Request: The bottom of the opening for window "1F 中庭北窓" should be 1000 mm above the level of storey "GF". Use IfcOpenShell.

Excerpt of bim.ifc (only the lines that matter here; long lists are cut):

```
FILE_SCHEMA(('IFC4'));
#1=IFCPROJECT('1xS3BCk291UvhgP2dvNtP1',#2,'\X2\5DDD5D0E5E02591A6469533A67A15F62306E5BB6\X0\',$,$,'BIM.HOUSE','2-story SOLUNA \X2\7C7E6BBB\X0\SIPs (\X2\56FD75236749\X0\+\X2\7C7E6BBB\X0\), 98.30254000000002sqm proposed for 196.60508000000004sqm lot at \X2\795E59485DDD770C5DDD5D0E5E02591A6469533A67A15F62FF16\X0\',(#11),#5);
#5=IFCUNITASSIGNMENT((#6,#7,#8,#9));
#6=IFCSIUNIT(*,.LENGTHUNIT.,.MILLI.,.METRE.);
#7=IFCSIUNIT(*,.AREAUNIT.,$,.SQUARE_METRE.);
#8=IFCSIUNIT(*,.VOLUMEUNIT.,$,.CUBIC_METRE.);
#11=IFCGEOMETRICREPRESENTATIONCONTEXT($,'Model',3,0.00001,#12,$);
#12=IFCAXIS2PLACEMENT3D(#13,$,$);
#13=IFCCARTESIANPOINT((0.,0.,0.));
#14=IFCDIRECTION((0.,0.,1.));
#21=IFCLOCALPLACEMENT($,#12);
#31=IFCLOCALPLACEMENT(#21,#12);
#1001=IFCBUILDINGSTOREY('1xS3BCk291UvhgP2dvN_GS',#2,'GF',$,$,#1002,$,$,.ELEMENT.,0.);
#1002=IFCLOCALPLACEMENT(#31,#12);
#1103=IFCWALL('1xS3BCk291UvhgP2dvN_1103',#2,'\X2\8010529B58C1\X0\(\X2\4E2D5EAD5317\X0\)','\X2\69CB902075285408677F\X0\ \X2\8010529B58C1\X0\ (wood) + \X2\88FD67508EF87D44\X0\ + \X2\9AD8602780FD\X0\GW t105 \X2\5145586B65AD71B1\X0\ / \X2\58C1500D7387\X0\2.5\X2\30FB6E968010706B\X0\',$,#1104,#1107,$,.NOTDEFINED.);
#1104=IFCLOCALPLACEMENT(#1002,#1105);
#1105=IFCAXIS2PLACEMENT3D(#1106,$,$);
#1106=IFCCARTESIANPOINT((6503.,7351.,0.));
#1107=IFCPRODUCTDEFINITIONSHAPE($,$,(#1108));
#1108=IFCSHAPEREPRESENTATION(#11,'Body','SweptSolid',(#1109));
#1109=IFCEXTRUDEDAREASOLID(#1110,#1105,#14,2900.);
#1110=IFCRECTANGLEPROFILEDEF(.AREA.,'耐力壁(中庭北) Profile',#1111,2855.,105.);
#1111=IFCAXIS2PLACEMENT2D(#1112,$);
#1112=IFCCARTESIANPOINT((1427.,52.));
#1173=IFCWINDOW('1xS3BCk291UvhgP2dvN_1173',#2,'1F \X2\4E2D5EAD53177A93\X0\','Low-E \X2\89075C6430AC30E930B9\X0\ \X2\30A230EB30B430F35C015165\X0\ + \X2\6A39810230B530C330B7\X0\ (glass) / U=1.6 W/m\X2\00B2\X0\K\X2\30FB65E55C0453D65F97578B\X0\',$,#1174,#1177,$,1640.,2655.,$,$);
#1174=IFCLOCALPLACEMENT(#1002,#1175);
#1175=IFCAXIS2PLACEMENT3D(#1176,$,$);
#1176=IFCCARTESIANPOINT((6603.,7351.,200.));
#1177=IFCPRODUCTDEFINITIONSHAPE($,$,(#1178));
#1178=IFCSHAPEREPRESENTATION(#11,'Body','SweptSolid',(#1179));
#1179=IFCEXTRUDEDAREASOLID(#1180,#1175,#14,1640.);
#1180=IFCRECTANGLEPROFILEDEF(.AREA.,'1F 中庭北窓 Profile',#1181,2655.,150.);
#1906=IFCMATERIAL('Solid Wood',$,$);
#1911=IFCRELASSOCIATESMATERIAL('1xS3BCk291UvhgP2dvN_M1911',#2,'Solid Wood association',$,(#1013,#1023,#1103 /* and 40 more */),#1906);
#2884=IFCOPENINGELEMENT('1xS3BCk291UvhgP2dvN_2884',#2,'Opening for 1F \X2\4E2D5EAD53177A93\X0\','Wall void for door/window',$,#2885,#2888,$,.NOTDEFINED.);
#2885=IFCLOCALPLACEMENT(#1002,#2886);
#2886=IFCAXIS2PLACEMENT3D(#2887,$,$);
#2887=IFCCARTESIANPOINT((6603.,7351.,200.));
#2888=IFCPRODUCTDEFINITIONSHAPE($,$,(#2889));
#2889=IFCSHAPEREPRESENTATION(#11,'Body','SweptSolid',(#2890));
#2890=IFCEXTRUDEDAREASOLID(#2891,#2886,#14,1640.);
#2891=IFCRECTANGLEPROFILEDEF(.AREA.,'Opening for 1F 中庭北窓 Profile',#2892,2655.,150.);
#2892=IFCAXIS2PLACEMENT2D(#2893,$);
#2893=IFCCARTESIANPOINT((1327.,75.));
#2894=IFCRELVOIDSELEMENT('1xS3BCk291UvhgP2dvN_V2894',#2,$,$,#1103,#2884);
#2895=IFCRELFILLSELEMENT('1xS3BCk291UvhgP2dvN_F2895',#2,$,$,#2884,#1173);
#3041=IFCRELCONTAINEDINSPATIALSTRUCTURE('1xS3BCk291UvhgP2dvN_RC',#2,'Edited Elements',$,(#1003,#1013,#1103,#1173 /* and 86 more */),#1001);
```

```python
import numpy as np
import ifcopenshell
import ifcopenshell.api.geometry
import ifcopenshell.geom
import ifcopenshell.util.element
import ifcopenshell.util.placement
import ifcopenshell.util.shape
import ifcopenshell.util.unit

model = ifcopenshell.open("bim.ifc")
unit_scale = ifcopenshell.util.unit.calculate_unit_scale(model)

window = model.by_guid("1xS3BCk291UvhgP2dvN_1173")
opening = window.FillsVoids[0].RelatingOpeningElement
storey = ifcopenshell.util.element.get_container(window, ifc_class="IfcBuildingStorey")
level = ifcopenshell.util.placement.get_local_placement(storey.ObjectPlacement)[2, 3]

# The opening's origin need not be at the sill, so measure its lowest point.
shape = ifcopenshell.geom.create_shape(ifcopenshell.geom.settings(), opening)
bottom = ifcopenshell.util.shape.get_shape_bottom_elevation(shape, shape.geometry) / unit_scale
dz = level + 1 / unit_scale - bottom

shift = np.array([0.0, 0.0, dz])
# The window is not placed relative to its opening, so move both.
for product in (opening, window):
    matrix = ifcopenshell.util.placement.get_local_placement(product.ObjectPlacement)
    matrix[:3, 3] += shift
    ifcopenshell.api.geometry.edit_object_placement(model, product=product, matrix=matrix, is_si=False)

print(f"moved by {dz * unit_scale:+.3f} m")

model.write("bim_edited.ifc")
```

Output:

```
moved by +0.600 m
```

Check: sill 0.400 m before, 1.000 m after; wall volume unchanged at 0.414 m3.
